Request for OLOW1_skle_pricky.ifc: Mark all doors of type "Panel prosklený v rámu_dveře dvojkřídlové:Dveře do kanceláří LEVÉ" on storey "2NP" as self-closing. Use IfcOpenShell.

First a look at what the model holds.

```python
import ifcopenshell
import ifcopenshell.util.element

model = ifcopenshell.open("OLOW1_skle_pricky.ifc")
print(model.schema)
storey = next(s for s in model.by_type("IfcBuildingStorey") if s.Name == "2NP")
doors = [e for e in ifcopenshell.util.element.get_decomposition(storey) if e.is_a("IfcDoor")]
seen = {}
for e in doors:
    element_type = ifcopenshell.util.element.get_type(e)
    key = (element_type.Name if element_type != e and element_type else None, ifcopenshell.util.element.get_pset(e, "Pset_DoorCommon", "SelfClosing"))
    seen[key] = seen.get(key, 0) + 1
for (name, value), count in sorted(seen.items(), key=str):
    print(count, "x", name, "|", value)
```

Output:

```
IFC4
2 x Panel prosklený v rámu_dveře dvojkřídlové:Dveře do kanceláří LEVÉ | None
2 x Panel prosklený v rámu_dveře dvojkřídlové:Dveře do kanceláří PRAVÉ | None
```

```python
import ifcopenshell
import ifcopenshell.api.pset
import ifcopenshell.util.element

model = ifcopenshell.open("OLOW1_skle_pricky.ifc")

storey = next(s for s in model.by_type("IfcBuildingStorey") if s.Name == "2NP")
doors = [e for e in ifcopenshell.util.element.get_decomposition(storey) if e.is_a("IfcDoor")]

count = 0
for e in doors:
    element_type = ifcopenshell.util.element.get_type(e)
    if element_type in (None, e) or element_type.Name != "Panel prosklený v rámu_dveře dvojkřídlové:Dveře do kanceláří LEVÉ":
        continue
    # add_pset returns the element's existing set when there is one.
    pset = ifcopenshell.api.pset.add_pset(model, product=e, name="Pset_DoorCommon")
    ifcopenshell.api.pset.edit_pset(model, pset=pset, properties={"SelfClosing": True})
    count += 1

print(count, "doors updated")

model.write("OLOW1_skle_pricky_v2.ifc")
```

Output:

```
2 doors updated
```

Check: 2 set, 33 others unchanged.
